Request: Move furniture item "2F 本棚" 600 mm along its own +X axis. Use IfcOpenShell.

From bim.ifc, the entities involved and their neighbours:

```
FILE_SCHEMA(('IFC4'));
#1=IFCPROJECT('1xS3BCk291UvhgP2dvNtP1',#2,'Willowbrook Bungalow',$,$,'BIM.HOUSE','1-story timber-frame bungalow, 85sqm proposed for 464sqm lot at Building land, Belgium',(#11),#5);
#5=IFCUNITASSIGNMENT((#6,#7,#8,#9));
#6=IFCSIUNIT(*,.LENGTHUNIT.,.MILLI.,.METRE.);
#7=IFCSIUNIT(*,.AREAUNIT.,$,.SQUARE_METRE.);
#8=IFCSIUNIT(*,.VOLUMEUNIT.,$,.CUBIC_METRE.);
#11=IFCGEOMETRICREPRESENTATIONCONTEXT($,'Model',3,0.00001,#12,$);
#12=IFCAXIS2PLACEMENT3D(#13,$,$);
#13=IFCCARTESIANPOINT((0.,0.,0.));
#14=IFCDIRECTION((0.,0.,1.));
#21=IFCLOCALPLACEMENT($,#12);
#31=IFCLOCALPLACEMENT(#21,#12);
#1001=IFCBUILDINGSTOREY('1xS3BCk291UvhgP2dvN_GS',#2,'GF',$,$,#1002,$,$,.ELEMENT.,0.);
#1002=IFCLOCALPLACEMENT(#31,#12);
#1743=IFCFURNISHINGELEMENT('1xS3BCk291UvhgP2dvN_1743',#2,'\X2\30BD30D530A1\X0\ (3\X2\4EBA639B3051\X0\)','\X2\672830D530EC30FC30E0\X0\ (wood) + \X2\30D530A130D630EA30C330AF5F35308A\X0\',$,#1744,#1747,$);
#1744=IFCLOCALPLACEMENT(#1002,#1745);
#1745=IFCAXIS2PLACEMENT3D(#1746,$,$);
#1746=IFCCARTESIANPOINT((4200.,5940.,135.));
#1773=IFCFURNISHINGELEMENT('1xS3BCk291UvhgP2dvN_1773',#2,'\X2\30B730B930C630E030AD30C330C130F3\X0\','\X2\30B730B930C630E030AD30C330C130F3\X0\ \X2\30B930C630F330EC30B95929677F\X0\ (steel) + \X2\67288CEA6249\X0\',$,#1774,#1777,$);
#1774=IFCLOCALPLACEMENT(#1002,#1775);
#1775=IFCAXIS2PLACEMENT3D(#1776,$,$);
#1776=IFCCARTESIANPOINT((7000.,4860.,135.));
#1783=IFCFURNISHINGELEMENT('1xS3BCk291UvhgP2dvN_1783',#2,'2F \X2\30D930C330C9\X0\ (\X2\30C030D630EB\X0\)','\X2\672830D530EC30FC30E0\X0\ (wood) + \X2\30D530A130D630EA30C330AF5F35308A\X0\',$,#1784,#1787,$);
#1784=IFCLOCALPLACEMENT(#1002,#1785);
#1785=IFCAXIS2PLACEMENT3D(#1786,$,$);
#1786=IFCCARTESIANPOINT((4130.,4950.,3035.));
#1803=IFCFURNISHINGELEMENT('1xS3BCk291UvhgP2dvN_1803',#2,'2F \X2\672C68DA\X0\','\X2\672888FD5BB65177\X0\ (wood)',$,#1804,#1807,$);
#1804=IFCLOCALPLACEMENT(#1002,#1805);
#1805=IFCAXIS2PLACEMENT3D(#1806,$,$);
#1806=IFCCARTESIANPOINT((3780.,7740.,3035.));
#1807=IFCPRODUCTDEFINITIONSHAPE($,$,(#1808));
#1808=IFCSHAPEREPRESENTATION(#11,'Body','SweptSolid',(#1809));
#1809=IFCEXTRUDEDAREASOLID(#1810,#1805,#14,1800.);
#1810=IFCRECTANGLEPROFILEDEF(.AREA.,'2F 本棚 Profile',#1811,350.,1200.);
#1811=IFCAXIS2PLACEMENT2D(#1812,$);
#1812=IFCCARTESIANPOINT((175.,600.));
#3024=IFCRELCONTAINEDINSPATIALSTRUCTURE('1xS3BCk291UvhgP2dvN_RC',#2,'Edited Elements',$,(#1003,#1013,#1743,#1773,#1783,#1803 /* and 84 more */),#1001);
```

```python
import ifcopenshell
import ifcopenshell.api.geometry
import ifcopenshell.util.placement

model = ifcopenshell.open("bim.ifc")

item = model.by_guid("1xS3BCk291UvhgP2dvN_1803")
matrix = ifcopenshell.util.placement.get_local_placement(item.ObjectPlacement)
matrix[:3, 3] += matrix[:3, 0] * 600.0
ifcopenshell.api.geometry.edit_object_placement(model, product=item, matrix=matrix, is_si=False)

print(ifcopenshell.util.placement.get_local_placement(item.ObjectPlacement).round(3) + 0.0)

model.write("bim_edited.ifc")
```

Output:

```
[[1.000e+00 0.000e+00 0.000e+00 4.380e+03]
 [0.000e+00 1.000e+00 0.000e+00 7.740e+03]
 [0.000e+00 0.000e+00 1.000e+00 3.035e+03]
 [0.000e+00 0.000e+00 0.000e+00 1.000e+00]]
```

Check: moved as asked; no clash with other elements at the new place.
